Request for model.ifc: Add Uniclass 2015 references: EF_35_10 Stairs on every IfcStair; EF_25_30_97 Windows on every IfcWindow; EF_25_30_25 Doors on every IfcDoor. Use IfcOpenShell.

First a look at what the model holds.

```python
import ifcopenshell

model = ifcopenshell.open("model.ifc")
print(model.schema)
print("classifications:", [c.Name for c in model.by_type("IfcClassification")])
for ifc_class in ("IfcDoor", "IfcRoof", "IfcStair", "IfcWall", "IfcWindow"):
    print(ifc_class, len(model.by_type(ifc_class)))
```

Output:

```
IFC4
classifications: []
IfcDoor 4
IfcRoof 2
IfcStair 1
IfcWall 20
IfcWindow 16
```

```python
import ifcopenshell
import ifcopenshell.api.classification

model = ifcopenshell.open("model.ifc")

system = ifcopenshell.api.classification.add_classification(model, classification="Uniclass 2015")

codes = {
    "IfcStair": ("EF_35_10", "Stairs"),
    "IfcWindow": ("EF_25_30_97", "Windows"),
    "IfcDoor": ("EF_25_30_25", "Doors"),
}
for ifc_class, (code, name) in codes.items():
    products = model.by_type(ifc_class)
    ifcopenshell.api.classification.add_reference(
        model, products=products, classification=system, identification=code, name=name
    )
    print(code, len(products))

model.write("model-out.ifc")
```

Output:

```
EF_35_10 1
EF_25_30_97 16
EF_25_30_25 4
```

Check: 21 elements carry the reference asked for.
